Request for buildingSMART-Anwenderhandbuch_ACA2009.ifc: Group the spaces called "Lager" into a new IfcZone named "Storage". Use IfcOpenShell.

First a look at what the model holds.

```python
import ifcopenshell

model = ifcopenshell.open("buildingSMART-Anwenderhandbuch_ACA2009.ifc")
print(model.schema)
seen = {}
for space in model.by_type("IfcSpace"):
    seen[space.LongName] = seen.get(space.LongName, 0) + 1
for name, count in sorted(seen.items(), key=str):
    print(count, "x", name)
print("zones:", [z.Name for z in model.by_type("IfcZone")][:20])
```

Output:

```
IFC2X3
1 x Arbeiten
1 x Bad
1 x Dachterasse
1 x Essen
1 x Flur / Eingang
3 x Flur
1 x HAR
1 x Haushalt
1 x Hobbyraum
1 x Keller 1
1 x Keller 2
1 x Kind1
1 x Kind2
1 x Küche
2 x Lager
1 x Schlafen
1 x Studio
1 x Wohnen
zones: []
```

```python
import ifcopenshell
import ifcopenshell.api.group
import ifcopenshell.api.root

model = ifcopenshell.open("buildingSMART-Anwenderhandbuch_ACA2009.ifc")

names = {"Lager"}
spaces = [s for s in model.by_type("IfcSpace") if s.LongName in names]

zone = ifcopenshell.api.root.create_entity(model, ifc_class="IfcZone", name="Storage")
ifcopenshell.api.group.assign_group(model, products=spaces, group=zone)
print(len(spaces), "spaces in", zone.Name)

model.write("buildingSMART-Anwenderhandbuch_ACA2009_v2.ifc")
```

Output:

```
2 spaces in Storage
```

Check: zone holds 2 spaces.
